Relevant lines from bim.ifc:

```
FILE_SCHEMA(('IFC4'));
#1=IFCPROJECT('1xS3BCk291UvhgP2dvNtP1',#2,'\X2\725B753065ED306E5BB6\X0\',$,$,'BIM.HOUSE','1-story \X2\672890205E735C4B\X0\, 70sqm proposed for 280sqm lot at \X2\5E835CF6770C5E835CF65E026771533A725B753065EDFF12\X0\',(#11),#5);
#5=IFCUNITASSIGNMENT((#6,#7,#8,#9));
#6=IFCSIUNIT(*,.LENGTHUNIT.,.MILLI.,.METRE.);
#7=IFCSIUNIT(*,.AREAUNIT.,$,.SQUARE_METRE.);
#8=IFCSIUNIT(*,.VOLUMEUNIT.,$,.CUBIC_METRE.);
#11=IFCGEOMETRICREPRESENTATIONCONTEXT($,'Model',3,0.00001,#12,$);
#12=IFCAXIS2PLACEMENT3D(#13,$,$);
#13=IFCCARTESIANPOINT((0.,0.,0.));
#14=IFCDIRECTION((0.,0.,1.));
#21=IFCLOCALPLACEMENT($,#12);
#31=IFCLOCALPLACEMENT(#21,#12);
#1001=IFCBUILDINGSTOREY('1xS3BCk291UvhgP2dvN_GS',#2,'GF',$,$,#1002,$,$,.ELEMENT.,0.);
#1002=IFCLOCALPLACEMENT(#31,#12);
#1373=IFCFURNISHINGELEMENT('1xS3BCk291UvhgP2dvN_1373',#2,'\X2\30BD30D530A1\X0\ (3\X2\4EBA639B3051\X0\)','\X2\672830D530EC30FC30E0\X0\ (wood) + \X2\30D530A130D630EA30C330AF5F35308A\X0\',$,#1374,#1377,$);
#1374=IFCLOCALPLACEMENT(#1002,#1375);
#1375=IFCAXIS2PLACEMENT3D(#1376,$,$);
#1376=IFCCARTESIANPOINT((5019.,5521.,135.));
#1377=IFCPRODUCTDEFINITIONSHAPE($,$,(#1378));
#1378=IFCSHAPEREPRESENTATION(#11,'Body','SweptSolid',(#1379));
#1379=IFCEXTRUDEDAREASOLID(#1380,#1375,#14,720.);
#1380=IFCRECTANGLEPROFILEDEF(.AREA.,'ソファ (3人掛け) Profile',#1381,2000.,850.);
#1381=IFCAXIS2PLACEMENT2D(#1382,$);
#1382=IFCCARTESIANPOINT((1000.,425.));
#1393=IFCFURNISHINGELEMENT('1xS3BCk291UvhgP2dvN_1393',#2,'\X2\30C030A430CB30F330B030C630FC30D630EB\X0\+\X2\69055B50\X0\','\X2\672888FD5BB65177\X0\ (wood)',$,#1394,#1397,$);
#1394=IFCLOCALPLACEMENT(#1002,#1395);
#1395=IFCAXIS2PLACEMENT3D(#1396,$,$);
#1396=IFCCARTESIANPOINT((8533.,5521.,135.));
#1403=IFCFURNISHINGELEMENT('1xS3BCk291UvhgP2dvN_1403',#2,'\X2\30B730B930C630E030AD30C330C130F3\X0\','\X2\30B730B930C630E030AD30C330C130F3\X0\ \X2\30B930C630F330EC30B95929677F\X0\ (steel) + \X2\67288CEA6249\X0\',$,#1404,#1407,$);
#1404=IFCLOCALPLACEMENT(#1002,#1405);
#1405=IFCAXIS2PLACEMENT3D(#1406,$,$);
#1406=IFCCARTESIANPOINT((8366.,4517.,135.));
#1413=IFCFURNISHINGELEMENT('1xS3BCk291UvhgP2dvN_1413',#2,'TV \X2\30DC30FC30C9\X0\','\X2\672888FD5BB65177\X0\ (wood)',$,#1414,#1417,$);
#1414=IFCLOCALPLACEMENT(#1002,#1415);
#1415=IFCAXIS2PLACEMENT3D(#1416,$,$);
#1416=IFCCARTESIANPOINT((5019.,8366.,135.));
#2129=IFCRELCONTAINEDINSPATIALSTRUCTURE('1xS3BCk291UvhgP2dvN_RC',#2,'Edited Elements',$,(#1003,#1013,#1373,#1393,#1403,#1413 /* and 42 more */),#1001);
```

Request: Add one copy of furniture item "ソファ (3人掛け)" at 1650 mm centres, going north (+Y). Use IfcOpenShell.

```python
import numpy as np
import ifcopenshell
import ifcopenshell.api.geometry
import ifcopenshell.api.root
import ifcopenshell.util.element
import ifcopenshell.util.placement
import ifcopenshell.util.unit

model = ifcopenshell.open("bim.ifc")
unit_scale = ifcopenshell.util.unit.calculate_unit_scale(model)


def reuse_history(source, copy):
    """copy_class also copies each property set's owner history, people and application; keep the originals."""
    for rel in copy.IsDefinedBy:
        if rel.is_a("IfcRelDefinesByProperties") and (history := rel.RelatingPropertyDefinition.OwnerHistory):
            rel.RelatingPropertyDefinition.OwnerHistory = source.OwnerHistory
            ifcopenshell.util.element.remove_deep2(model, history)


source = model.by_guid("1xS3BCk291UvhgP2dvN_1373")
base = ifcopenshell.util.placement.get_local_placement(source.ObjectPlacement)
step = np.array([0.0, 1.0, 0.0]) * 1.65 / unit_scale

for i in range(1, 2):
    copy = ifcopenshell.api.root.copy_class(model, product=source)
    copy.Representation = ifcopenshell.util.element.copy_deep(
        model, source.Representation, exclude=["IfcGeometricRepresentationContext", "IfcRepresentationMap"]
    )
    reuse_history(source, copy)
    matrix = base.copy()
    matrix[:3, 3] += i * step
    print("added at", matrix[:3, 3].round(3) + 0.0)
    ifcopenshell.api.geometry.edit_object_placement(model, product=copy, matrix=matrix, is_si=False)

model.write("bim_rev.ifc")
```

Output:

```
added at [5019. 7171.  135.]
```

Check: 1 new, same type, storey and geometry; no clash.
